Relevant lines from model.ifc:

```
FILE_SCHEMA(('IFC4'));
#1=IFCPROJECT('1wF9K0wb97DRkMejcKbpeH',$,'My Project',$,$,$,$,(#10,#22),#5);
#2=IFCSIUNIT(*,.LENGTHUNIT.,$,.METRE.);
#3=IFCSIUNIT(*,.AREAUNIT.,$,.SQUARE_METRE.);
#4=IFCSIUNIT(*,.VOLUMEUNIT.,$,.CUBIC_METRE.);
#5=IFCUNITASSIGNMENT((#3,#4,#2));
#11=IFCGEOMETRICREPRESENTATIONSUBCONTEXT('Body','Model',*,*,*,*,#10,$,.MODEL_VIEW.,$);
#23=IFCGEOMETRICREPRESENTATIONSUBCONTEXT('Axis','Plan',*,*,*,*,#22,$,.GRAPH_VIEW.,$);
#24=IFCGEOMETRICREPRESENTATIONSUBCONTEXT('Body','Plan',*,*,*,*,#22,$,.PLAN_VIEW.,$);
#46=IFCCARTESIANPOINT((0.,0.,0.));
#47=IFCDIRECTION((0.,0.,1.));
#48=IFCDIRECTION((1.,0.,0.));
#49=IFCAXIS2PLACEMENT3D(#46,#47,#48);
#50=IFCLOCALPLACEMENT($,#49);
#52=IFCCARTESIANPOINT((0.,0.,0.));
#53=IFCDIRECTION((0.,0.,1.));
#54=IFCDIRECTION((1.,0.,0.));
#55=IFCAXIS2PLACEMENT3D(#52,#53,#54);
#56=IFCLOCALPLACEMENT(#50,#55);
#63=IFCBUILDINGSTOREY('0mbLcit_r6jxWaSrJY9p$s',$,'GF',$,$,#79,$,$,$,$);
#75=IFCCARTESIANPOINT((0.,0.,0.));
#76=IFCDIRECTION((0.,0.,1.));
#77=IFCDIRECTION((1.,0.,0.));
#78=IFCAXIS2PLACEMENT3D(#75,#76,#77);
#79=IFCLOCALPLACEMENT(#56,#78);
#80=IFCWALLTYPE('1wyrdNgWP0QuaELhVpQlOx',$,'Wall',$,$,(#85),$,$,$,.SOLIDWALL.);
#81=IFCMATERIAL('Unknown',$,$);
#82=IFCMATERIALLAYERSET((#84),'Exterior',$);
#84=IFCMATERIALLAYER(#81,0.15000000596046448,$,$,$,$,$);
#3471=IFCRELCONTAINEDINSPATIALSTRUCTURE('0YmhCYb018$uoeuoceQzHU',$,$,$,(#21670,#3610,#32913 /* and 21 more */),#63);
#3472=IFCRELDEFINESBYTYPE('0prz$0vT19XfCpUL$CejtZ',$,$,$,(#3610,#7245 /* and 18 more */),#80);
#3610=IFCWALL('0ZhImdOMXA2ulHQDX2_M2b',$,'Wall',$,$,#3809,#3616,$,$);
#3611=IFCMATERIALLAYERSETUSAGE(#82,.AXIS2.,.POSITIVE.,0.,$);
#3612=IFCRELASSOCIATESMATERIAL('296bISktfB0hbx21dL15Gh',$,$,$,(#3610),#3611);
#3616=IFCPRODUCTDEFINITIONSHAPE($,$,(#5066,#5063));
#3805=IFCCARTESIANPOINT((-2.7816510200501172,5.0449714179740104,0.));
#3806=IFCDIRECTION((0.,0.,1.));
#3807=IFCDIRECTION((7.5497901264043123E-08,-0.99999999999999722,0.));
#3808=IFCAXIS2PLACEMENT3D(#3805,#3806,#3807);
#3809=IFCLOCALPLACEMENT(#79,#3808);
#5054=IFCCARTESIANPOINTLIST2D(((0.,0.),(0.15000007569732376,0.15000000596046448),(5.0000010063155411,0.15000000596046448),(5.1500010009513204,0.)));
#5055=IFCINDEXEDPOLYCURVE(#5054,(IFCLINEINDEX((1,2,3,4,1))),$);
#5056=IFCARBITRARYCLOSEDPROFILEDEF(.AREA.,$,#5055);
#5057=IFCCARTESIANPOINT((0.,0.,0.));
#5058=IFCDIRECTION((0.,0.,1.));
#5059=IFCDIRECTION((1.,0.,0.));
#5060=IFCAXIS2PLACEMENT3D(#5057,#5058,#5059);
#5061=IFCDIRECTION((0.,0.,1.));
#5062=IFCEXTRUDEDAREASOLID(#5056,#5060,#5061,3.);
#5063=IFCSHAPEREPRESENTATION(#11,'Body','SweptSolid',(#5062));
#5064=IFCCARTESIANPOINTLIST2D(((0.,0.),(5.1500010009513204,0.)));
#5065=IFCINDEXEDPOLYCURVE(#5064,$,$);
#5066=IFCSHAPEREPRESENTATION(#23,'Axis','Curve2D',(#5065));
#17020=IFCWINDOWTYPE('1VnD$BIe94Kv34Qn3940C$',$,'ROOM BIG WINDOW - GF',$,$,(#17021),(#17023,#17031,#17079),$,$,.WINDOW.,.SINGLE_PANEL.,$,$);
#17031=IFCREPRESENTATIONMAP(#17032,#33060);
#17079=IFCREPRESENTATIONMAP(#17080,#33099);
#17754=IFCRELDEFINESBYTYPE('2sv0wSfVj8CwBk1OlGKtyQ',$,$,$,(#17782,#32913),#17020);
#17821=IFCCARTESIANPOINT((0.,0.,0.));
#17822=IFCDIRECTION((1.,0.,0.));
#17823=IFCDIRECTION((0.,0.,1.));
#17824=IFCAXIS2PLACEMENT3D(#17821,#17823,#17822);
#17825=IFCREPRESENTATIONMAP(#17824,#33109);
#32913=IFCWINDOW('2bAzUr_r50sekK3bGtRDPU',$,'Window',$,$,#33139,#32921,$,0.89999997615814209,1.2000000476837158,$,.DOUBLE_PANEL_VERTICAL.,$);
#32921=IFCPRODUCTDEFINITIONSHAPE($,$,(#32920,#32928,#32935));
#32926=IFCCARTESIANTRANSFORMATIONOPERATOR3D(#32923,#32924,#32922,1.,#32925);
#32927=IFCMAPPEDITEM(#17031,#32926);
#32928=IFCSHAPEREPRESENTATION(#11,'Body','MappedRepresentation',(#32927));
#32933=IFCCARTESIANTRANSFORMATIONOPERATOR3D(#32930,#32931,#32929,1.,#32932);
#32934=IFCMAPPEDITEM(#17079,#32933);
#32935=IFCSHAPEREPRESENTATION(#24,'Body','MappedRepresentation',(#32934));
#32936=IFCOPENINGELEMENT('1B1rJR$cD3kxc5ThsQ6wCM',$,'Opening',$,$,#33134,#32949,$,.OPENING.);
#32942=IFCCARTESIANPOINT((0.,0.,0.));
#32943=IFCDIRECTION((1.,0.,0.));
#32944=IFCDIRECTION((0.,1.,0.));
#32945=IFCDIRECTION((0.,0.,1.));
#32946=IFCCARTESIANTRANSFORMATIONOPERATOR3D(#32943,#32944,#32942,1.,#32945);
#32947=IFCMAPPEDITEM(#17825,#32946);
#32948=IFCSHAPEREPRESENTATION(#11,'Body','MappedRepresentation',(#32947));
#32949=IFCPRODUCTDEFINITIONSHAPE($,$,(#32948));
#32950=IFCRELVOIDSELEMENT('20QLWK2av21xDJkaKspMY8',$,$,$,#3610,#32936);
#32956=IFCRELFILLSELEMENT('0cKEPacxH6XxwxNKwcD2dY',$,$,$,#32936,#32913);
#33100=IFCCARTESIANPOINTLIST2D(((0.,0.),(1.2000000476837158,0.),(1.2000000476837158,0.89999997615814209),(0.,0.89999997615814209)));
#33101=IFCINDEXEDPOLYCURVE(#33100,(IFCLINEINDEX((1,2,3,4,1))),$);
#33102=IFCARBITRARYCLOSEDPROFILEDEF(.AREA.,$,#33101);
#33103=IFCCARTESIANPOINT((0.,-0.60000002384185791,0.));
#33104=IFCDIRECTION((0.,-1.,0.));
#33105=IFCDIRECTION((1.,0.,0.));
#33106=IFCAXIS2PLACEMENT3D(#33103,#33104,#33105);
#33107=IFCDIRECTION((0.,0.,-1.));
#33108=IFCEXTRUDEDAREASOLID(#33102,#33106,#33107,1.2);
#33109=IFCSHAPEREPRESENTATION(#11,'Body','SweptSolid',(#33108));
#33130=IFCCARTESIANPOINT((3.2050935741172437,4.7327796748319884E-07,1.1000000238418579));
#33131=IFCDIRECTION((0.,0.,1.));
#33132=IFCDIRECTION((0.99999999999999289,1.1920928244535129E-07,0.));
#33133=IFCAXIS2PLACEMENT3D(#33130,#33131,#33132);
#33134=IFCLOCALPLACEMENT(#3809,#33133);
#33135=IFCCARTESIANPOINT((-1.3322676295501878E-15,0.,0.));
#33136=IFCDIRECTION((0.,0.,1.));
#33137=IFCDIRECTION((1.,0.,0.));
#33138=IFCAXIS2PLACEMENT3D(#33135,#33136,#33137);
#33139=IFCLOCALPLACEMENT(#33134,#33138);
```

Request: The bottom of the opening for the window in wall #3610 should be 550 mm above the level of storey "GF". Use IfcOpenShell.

```python
import numpy as np
import ifcopenshell
import ifcopenshell.api.geometry
import ifcopenshell.geom
import ifcopenshell.util.element
import ifcopenshell.util.placement
import ifcopenshell.util.shape
import ifcopenshell.util.unit

model = ifcopenshell.open("model.ifc")
unit_scale = ifcopenshell.util.unit.calculate_unit_scale(model)

window = model.by_guid("2bAzUr_r50sekK3bGtRDPU")
opening = window.FillsVoids[0].RelatingOpeningElement
storey = ifcopenshell.util.element.get_container(window, ifc_class="IfcBuildingStorey")
level = ifcopenshell.util.placement.get_local_placement(storey.ObjectPlacement)[2, 3]

# The opening's origin need not be at the sill, so measure its lowest point.
shape = ifcopenshell.geom.create_shape(ifcopenshell.geom.settings(), opening)
bottom = ifcopenshell.util.shape.get_shape_bottom_elevation(shape, shape.geometry) / unit_scale
dz = level + 0.55 - bottom

shift = np.array([0.0, 0.0, dz])
# The window is placed relative to its opening, so it follows when the opening moves.
matrix = ifcopenshell.util.placement.get_local_placement(opening.ObjectPlacement)
matrix[:3, 3] += shift
ifcopenshell.api.geometry.edit_object_placement(
    model, product=opening, matrix=matrix, is_si=False, should_transform_children=True
)

print(f"moved by {dz * unit_scale:+.3f} m")

model.write("model-out.ifc")
```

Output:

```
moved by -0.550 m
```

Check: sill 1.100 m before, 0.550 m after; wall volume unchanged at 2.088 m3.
